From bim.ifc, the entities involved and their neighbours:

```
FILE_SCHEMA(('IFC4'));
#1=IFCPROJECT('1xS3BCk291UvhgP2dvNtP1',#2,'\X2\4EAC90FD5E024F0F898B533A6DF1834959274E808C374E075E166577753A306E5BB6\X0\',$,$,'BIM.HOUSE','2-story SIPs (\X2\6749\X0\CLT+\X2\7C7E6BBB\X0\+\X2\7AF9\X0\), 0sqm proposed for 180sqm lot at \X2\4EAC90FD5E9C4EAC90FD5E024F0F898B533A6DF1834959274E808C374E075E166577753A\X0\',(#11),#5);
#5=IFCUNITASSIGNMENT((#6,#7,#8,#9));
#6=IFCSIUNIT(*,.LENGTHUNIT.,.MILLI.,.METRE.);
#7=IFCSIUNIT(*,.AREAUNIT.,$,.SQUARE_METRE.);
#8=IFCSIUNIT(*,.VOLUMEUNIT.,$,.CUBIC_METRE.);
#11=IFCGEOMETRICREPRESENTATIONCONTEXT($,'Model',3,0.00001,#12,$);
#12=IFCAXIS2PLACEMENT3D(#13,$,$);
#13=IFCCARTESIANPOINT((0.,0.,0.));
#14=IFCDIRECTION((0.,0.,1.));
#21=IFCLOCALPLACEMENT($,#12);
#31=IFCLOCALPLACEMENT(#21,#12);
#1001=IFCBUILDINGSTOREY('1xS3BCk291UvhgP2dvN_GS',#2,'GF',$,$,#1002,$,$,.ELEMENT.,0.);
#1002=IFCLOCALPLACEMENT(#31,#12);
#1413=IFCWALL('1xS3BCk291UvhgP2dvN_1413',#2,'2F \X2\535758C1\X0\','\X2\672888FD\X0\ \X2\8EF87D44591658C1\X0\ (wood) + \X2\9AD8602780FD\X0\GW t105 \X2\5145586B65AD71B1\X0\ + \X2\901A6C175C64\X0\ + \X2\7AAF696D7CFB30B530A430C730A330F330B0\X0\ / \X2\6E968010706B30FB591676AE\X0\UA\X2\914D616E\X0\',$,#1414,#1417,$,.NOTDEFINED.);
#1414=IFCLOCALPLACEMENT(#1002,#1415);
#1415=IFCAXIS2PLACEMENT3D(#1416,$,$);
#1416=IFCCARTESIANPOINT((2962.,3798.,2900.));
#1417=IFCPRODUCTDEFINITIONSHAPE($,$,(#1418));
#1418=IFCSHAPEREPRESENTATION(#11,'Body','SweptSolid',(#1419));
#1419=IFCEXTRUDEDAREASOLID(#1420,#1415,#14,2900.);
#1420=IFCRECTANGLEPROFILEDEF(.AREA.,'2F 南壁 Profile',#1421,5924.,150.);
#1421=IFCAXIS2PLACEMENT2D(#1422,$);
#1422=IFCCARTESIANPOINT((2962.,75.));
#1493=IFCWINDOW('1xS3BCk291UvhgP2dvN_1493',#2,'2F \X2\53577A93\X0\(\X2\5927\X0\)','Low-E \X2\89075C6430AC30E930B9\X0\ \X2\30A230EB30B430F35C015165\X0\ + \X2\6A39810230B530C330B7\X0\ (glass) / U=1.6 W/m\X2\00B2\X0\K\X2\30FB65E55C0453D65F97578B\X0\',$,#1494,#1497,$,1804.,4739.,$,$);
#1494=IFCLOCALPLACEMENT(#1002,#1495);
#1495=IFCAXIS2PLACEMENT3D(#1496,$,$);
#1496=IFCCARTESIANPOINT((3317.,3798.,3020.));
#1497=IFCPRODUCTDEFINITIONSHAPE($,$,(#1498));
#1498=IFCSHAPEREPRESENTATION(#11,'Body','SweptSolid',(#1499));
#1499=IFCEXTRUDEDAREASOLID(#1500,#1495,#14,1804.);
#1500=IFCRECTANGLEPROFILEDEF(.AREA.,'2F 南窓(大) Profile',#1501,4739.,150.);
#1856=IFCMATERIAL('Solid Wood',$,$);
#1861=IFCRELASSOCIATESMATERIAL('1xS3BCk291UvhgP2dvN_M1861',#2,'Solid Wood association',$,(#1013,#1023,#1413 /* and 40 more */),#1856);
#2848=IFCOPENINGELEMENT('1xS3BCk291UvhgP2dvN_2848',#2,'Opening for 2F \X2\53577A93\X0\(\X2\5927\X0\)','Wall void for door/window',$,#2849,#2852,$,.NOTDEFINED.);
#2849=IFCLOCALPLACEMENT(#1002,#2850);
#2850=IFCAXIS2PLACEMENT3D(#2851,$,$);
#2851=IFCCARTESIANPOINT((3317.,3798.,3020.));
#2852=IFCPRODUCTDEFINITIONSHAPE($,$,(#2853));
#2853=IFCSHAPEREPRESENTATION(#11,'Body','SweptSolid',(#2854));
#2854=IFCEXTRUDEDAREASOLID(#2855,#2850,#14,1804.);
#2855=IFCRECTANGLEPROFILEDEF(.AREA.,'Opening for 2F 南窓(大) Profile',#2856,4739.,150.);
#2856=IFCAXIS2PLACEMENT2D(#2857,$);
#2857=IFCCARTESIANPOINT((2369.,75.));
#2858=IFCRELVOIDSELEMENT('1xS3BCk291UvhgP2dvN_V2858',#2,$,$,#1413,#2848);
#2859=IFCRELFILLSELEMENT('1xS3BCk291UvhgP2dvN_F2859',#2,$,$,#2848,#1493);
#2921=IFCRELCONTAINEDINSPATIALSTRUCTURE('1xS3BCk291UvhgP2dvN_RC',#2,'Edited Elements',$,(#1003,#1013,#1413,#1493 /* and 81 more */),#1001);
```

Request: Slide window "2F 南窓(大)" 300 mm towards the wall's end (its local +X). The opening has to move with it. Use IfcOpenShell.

```python
import ifcopenshell
import ifcopenshell.api.geometry
import ifcopenshell.util.placement

model = ifcopenshell.open("bim.ifc")

window = model.by_guid("1xS3BCk291UvhgP2dvN_1493")
opening = window.FillsVoids[0].RelatingOpeningElement
wall = opening.VoidsElements[0].RelatingBuildingElement

wall_matrix = ifcopenshell.util.placement.get_local_placement(wall.ObjectPlacement)
shift = wall_matrix[:3, 0] * 300.0
before = ifcopenshell.util.placement.get_local_placement(window.ObjectPlacement)[:3, 3].copy()

# The window is not placed relative to its opening, so move both.
for product in (opening, window):
    matrix = ifcopenshell.util.placement.get_local_placement(product.ObjectPlacement)
    matrix[:3, 3] += shift
    ifcopenshell.api.geometry.edit_object_placement(model, product=product, matrix=matrix, is_si=False)

after = ifcopenshell.util.placement.get_local_placement(window.ObjectPlacement)[:3, 3]
print("window moved by", (after - before).round(3) + 0.0)

model.write("bim_updated.ifc")
```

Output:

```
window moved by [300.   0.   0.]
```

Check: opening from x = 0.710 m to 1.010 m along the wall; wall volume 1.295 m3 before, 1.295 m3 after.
